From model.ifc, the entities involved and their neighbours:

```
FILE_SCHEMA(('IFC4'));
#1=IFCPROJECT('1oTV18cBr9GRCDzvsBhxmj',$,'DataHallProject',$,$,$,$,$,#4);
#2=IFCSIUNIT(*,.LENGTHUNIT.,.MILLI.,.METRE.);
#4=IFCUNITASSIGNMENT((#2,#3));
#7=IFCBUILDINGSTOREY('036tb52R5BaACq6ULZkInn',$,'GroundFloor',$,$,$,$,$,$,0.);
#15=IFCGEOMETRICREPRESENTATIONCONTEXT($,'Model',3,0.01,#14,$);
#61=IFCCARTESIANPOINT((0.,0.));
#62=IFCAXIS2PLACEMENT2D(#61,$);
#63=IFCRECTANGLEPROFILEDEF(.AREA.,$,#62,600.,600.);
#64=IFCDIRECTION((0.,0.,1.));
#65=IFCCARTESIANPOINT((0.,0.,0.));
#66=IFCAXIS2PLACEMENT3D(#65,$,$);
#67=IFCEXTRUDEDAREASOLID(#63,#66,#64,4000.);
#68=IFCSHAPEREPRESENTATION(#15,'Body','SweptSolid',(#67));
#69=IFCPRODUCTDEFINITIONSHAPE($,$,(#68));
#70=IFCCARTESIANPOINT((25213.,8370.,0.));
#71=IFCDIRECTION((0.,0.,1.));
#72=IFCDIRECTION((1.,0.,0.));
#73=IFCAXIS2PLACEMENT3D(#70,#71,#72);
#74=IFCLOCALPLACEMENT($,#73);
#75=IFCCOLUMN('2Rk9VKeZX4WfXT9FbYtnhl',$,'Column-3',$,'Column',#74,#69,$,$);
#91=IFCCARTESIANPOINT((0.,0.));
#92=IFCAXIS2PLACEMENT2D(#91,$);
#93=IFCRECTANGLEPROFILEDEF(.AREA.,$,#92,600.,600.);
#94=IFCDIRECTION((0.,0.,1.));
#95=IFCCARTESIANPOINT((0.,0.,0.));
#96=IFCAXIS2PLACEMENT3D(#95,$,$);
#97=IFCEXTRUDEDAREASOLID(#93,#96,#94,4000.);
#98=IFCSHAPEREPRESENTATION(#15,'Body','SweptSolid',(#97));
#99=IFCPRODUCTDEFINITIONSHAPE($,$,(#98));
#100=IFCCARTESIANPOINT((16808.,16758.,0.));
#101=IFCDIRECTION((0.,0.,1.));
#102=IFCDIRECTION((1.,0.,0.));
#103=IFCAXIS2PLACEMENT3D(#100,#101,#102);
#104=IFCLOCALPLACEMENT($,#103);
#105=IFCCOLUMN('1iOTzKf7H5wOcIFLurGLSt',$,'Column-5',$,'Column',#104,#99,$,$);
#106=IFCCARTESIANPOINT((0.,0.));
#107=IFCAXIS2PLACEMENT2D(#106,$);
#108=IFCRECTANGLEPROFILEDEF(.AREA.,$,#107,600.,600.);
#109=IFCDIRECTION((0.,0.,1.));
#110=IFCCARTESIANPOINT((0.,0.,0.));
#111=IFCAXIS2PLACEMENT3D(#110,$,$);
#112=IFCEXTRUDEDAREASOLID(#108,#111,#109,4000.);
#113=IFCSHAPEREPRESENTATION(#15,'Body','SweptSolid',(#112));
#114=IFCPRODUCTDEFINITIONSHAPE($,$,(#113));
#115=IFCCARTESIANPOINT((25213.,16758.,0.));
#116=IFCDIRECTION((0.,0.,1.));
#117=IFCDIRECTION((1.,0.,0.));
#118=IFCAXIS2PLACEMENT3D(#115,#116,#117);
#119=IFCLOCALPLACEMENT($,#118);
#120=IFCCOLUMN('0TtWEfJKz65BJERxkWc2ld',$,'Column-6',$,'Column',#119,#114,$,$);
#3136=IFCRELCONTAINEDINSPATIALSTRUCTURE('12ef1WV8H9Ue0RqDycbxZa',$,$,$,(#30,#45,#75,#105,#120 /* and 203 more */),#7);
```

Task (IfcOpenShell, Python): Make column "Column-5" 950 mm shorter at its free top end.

```python
import ifcopenshell
import ifcopenshell.util.unit

model = ifcopenshell.open("model.ifc")
unit_scale = ifcopenshell.util.unit.calculate_unit_scale(model)

member = model.by_guid("1iOTzKf7H5wOcIFLurGLSt")
change = -0.95 / unit_scale

# The extrusion runs towards the end named, so only its depth changes.
body = next(r for r in member.Representation.Representations if r.RepresentationIdentifier == "Body")
solid = body.Items[0]
old_length = solid.Depth
solid.Depth += change

print(f"length {old_length:g} -> {solid.Depth:g}")

model.write("model_updated.ifc")
```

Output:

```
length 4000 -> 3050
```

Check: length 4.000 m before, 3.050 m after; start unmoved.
